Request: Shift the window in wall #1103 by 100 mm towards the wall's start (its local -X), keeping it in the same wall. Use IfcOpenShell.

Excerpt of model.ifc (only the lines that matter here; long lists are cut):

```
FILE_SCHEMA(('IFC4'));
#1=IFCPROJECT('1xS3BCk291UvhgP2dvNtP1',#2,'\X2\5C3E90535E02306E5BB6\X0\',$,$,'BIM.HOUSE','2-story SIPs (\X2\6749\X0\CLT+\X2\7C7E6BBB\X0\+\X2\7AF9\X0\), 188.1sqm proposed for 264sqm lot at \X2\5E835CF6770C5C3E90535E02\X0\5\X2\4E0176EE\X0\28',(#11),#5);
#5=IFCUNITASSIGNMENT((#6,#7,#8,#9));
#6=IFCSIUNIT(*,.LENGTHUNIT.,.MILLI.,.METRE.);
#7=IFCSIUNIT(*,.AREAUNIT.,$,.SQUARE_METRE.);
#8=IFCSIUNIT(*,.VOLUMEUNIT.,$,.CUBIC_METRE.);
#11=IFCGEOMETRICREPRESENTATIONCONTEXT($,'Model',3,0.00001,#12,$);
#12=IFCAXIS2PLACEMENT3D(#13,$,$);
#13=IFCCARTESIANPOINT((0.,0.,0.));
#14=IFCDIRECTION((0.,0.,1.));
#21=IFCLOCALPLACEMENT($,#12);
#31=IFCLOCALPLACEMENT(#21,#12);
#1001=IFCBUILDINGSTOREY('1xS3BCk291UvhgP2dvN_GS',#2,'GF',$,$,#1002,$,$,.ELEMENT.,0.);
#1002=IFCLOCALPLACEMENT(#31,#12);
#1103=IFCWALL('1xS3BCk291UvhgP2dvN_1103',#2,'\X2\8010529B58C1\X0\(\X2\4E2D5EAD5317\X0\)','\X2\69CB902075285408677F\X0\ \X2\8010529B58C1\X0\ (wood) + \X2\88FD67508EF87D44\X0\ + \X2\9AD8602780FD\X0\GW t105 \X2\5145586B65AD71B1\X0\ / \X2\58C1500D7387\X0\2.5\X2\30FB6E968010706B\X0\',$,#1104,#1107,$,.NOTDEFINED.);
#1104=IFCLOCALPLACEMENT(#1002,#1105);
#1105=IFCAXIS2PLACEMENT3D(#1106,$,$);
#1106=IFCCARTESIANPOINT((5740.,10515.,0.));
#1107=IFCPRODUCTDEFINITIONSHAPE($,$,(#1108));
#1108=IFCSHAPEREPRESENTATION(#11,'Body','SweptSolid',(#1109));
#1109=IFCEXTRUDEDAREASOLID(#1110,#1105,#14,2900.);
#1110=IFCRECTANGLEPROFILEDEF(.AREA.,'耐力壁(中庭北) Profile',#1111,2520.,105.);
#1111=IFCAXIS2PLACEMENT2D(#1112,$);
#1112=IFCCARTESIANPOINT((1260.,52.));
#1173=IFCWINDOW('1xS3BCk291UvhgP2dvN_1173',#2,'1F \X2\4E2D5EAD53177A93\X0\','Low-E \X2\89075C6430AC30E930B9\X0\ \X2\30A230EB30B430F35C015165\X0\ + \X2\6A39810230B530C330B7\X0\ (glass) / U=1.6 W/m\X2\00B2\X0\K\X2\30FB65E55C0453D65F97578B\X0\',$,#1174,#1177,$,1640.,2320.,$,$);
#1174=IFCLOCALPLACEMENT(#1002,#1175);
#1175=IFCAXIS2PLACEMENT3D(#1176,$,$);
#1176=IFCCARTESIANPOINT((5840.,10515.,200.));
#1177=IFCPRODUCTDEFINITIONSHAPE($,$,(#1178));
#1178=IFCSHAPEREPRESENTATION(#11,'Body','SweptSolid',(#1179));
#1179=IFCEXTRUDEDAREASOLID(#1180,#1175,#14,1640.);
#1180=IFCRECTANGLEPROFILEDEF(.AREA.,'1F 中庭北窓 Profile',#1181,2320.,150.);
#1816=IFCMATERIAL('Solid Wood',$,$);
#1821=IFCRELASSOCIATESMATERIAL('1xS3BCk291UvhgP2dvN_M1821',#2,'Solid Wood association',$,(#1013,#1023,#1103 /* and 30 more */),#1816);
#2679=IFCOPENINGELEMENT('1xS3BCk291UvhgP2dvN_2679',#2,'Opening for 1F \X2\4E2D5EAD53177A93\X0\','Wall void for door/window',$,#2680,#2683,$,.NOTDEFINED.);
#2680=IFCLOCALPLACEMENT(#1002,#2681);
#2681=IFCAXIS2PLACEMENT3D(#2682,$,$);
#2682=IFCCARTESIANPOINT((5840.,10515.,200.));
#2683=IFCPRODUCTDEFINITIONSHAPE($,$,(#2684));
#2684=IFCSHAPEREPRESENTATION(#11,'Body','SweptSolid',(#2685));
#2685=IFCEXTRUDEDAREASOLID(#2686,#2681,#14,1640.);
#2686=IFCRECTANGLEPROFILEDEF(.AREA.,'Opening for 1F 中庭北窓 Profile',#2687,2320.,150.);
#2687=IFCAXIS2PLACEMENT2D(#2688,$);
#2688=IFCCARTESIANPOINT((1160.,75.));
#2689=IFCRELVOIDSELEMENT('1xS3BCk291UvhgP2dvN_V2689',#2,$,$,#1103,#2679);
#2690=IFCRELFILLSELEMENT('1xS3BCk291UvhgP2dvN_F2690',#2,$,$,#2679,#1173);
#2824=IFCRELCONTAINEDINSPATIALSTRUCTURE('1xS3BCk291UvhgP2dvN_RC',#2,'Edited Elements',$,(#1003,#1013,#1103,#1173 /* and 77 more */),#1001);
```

```python
import ifcopenshell
import ifcopenshell.api.geometry
import ifcopenshell.util.placement
import ifcopenshell.util.unit

model = ifcopenshell.open("model.ifc")
unit_scale = ifcopenshell.util.unit.calculate_unit_scale(model)

window = model.by_id(1173)
opening = window.FillsVoids[0].RelatingOpeningElement
wall = opening.VoidsElements[0].RelatingBuildingElement

wall_matrix = ifcopenshell.util.placement.get_local_placement(wall.ObjectPlacement)
shift = wall_matrix[:3, 0] * -0.1 / unit_scale
before = ifcopenshell.util.placement.get_local_placement(window.ObjectPlacement)[:3, 3].copy()

# The window is not placed relative to its opening, so move both.
for product in (opening, window):
    matrix = ifcopenshell.util.placement.get_local_placement(product.ObjectPlacement)
    matrix[:3, 3] += shift
    ifcopenshell.api.geometry.edit_object_placement(model, product=product, matrix=matrix, is_si=False)

after = ifcopenshell.util.placement.get_local_placement(window.ObjectPlacement)[:3, 3]
print("window moved by", (after - before).round(3) + 0.0)

model.write("model_v2.ifc")
```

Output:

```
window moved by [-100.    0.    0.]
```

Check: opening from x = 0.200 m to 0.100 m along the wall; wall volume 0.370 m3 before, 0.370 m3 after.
